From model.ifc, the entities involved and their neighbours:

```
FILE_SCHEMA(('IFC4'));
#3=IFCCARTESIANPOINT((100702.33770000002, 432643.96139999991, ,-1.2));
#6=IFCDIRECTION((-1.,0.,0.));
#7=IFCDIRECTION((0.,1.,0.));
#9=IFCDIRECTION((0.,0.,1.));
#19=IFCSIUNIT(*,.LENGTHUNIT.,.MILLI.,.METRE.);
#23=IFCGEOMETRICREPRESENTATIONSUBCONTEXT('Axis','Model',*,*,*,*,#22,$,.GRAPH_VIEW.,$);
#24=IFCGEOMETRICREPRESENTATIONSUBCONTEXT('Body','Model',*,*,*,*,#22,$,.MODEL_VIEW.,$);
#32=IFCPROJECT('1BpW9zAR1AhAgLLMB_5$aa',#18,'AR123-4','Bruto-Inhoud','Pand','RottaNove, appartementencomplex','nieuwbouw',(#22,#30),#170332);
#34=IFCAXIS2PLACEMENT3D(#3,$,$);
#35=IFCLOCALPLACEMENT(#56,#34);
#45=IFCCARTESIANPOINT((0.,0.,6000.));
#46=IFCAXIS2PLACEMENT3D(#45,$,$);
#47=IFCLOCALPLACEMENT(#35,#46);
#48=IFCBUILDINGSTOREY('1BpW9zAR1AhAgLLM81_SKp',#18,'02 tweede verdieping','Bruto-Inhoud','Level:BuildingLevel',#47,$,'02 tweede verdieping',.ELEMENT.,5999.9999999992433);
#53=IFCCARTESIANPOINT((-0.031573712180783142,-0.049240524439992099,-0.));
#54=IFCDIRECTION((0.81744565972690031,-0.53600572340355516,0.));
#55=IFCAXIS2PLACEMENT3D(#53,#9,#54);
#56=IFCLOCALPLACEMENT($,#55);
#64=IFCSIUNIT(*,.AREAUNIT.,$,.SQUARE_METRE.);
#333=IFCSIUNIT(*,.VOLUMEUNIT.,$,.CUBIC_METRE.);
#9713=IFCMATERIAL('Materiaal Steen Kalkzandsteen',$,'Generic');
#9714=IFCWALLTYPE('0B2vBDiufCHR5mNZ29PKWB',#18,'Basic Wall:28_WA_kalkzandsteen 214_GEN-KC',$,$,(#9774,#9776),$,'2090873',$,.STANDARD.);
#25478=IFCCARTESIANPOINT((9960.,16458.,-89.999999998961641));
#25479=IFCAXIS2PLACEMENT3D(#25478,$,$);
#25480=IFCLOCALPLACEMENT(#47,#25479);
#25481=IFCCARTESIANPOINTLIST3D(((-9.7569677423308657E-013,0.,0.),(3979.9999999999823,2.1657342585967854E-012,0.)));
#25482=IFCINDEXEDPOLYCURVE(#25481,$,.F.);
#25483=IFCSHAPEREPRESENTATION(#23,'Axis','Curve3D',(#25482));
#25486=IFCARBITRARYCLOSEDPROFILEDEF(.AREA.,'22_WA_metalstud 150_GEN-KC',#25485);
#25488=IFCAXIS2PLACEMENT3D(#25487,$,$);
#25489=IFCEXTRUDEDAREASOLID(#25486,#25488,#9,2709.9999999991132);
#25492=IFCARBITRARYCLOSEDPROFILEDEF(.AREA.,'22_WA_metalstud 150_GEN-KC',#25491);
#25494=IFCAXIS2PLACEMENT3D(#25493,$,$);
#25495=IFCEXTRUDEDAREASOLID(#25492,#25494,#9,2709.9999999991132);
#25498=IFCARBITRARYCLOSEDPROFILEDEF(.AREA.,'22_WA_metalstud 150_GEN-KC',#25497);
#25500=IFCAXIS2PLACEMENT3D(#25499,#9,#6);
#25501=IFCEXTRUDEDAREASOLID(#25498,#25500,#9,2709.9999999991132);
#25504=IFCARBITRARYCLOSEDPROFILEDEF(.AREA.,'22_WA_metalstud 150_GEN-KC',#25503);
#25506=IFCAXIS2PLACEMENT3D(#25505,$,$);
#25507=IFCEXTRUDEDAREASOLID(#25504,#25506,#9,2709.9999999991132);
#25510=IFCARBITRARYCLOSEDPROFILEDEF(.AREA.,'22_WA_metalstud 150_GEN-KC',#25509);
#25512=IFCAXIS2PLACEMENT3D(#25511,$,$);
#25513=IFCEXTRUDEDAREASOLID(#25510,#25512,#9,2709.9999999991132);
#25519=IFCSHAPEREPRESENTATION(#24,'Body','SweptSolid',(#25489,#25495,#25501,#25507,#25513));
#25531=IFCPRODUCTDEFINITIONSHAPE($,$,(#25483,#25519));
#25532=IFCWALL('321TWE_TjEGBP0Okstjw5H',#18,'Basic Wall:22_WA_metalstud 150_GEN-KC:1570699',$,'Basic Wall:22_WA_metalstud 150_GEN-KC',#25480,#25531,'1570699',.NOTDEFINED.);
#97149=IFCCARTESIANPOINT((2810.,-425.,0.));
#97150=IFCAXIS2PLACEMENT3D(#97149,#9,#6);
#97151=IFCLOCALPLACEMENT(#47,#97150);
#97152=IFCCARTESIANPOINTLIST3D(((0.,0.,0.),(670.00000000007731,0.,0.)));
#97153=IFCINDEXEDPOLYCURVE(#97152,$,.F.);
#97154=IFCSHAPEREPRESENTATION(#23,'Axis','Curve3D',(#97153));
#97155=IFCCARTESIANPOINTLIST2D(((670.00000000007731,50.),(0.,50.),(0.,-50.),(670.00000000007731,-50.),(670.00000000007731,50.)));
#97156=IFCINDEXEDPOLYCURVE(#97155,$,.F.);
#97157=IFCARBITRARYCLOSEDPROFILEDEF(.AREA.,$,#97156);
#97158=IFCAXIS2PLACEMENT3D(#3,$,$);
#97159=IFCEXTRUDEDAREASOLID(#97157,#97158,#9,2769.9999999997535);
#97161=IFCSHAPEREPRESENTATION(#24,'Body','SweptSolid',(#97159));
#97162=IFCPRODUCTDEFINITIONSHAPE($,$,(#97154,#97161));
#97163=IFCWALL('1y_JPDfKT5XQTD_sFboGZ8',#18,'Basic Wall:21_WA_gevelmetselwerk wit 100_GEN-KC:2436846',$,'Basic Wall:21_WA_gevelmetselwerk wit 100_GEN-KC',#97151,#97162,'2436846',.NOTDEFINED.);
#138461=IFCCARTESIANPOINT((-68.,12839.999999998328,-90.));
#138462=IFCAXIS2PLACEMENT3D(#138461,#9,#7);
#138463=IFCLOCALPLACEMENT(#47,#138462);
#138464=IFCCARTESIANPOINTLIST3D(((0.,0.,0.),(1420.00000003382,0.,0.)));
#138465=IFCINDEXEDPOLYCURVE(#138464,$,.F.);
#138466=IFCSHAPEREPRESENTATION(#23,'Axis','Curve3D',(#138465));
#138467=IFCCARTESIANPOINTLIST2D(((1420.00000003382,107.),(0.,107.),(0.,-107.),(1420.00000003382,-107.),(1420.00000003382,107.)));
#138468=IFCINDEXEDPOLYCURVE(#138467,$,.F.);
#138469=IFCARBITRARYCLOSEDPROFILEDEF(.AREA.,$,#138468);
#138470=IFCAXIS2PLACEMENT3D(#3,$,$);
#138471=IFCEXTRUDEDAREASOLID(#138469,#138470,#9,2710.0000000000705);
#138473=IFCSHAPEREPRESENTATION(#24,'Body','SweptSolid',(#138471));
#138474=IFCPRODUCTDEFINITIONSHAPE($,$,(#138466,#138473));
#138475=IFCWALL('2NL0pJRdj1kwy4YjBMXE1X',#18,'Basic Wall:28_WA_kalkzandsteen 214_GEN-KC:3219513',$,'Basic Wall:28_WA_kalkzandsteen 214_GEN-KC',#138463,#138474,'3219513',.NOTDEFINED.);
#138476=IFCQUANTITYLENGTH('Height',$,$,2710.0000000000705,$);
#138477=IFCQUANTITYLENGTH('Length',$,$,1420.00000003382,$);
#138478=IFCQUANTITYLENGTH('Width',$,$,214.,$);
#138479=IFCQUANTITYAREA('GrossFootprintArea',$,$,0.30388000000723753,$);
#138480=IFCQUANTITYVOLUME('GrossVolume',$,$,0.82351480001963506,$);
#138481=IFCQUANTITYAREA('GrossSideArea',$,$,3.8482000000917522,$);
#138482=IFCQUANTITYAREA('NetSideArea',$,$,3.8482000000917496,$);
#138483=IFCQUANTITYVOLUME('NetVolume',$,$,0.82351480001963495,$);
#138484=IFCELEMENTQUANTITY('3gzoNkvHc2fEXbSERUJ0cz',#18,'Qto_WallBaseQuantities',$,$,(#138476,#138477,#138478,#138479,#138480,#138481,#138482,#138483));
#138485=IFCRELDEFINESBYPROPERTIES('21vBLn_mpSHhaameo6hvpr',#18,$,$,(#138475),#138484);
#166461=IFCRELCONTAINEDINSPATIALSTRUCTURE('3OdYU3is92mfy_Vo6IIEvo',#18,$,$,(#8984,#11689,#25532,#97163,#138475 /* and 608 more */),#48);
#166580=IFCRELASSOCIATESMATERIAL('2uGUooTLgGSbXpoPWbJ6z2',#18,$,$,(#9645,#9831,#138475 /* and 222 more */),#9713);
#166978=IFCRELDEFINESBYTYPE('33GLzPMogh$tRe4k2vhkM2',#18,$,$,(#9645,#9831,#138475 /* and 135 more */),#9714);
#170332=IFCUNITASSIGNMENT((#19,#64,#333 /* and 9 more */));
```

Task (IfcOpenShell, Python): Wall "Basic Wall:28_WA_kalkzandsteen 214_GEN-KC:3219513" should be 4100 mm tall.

```python
import ifcopenshell
import ifcopenshell.api.pset
import ifcopenshell.geom
import ifcopenshell.util.element
import ifcopenshell.util.representation
import ifcopenshell.util.shape
import ifcopenshell.util.unit

model = ifcopenshell.open("model.ifc")
unit_scale = ifcopenshell.util.unit.calculate_unit_scale(model)
area_scale = ifcopenshell.util.unit.calculate_unit_scale(model, "AREAUNIT")
volume_scale = ifcopenshell.util.unit.calculate_unit_scale(model, "VOLUMEUNIT")
settings = ifcopenshell.geom.settings()


def volume(element):
    """Net volume in cubic metres, openings subtracted."""
    shape = ifcopenshell.geom.create_shape(settings, element)
    return ifcopenshell.util.shape.get_volume(shape.geometry)


wall = model.by_guid("2NL0pJRdj1kwy4YjBMXE1X")
before = volume(wall)

body = ifcopenshell.util.representation.get_representation(wall, "Model", "Body")
solid = body.Items[0]
old_height = solid.Depth
solid.Depth = 4100.0
after = volume(wall)
thickness = 0.214  # wall thickness in metres

# Update the stored height, areas and volumes.
qto = model.by_id(ifcopenshell.util.element.get_pset(wall, "Qto_WallBaseQuantities", should_inherit=False)["id"])
ifcopenshell.api.pset.edit_qto(model, qto=qto, properties={
    "Height": solid.Depth,
    "GrossVolume": ifcopenshell.util.element.get_pset(wall, "Qto_WallBaseQuantities", "GrossVolume") * solid.Depth / old_height,
    "GrossSideArea": ifcopenshell.util.element.get_pset(wall, "Qto_WallBaseQuantities", "GrossSideArea") * solid.Depth / old_height,
    "NetSideArea": after / thickness / area_scale,
    "NetVolume": after / volume_scale,
})

print(f"height {old_height:g} -> {solid.Depth:g}, volume {before:.3f} -> {after:.3f} m3")

model.write("model_v2.ifc")
```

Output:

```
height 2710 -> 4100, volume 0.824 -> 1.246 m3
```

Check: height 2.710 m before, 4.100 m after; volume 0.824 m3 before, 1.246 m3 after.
